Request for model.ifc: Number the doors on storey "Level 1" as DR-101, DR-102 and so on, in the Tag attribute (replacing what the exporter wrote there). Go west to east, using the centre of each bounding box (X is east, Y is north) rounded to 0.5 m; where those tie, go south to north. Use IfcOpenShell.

First a look at what the model holds.

```python
import ifcopenshell
import ifcopenshell.util.element
import ifcopenshell.util.placement

model = ifcopenshell.open("model.ifc")
print(model.schema)
storey = next(s for s in model.by_type("IfcBuildingStorey") if s.Name == "Level 1")
doors = [e for e in ifcopenshell.util.element.get_decomposition(storey) if e.is_a("IfcDoor")]
for e in sorted(doors, key=lambda e: e.id()):
    origin = ifcopenshell.util.placement.get_local_placement(e.ObjectPlacement)[:3, 3]
    print(e.id(), e.Tag, e.Name, origin.round(2) + 0.0, sep=" | ")
```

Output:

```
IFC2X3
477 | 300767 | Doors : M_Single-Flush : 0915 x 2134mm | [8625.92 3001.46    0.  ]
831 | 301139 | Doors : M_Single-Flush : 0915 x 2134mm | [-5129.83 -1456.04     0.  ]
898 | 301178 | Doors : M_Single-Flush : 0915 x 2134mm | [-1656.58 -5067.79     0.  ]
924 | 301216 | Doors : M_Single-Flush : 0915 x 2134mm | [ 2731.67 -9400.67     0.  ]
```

```python
import ifcopenshell
import ifcopenshell.geom
import ifcopenshell.util.element
import ifcopenshell.util.shape

model = ifcopenshell.open("model.ifc")
settings = ifcopenshell.geom.settings()
settings.set("use-world-coords", True)


def centre(element):
    shape = ifcopenshell.geom.create_shape(settings, element)
    return ifcopenshell.util.shape.get_bbox_centroid(shape.geometry)


storey = next(s for s in model.by_type("IfcBuildingStorey") if s.Name == "Level 1")
doors = [e for e in ifcopenshell.util.element.get_decomposition(storey) if e.is_a("IfcDoor")]

# Insertion points can sit at a corner or the storey origin, so sort by the geometry (in metres).
centres = {e: centre(e) for e in doors}
doors.sort(key=lambda e: (round(centres[e][0] / 0.5), centres[e][1]))

for i, e in enumerate(doors, start=1):
    number = f"DR-1{i:02d}"
    e.Tag = number
    print(e.id(), number)

model.write("model_edited.ifc")
```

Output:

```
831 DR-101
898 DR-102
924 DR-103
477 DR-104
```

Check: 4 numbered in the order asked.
